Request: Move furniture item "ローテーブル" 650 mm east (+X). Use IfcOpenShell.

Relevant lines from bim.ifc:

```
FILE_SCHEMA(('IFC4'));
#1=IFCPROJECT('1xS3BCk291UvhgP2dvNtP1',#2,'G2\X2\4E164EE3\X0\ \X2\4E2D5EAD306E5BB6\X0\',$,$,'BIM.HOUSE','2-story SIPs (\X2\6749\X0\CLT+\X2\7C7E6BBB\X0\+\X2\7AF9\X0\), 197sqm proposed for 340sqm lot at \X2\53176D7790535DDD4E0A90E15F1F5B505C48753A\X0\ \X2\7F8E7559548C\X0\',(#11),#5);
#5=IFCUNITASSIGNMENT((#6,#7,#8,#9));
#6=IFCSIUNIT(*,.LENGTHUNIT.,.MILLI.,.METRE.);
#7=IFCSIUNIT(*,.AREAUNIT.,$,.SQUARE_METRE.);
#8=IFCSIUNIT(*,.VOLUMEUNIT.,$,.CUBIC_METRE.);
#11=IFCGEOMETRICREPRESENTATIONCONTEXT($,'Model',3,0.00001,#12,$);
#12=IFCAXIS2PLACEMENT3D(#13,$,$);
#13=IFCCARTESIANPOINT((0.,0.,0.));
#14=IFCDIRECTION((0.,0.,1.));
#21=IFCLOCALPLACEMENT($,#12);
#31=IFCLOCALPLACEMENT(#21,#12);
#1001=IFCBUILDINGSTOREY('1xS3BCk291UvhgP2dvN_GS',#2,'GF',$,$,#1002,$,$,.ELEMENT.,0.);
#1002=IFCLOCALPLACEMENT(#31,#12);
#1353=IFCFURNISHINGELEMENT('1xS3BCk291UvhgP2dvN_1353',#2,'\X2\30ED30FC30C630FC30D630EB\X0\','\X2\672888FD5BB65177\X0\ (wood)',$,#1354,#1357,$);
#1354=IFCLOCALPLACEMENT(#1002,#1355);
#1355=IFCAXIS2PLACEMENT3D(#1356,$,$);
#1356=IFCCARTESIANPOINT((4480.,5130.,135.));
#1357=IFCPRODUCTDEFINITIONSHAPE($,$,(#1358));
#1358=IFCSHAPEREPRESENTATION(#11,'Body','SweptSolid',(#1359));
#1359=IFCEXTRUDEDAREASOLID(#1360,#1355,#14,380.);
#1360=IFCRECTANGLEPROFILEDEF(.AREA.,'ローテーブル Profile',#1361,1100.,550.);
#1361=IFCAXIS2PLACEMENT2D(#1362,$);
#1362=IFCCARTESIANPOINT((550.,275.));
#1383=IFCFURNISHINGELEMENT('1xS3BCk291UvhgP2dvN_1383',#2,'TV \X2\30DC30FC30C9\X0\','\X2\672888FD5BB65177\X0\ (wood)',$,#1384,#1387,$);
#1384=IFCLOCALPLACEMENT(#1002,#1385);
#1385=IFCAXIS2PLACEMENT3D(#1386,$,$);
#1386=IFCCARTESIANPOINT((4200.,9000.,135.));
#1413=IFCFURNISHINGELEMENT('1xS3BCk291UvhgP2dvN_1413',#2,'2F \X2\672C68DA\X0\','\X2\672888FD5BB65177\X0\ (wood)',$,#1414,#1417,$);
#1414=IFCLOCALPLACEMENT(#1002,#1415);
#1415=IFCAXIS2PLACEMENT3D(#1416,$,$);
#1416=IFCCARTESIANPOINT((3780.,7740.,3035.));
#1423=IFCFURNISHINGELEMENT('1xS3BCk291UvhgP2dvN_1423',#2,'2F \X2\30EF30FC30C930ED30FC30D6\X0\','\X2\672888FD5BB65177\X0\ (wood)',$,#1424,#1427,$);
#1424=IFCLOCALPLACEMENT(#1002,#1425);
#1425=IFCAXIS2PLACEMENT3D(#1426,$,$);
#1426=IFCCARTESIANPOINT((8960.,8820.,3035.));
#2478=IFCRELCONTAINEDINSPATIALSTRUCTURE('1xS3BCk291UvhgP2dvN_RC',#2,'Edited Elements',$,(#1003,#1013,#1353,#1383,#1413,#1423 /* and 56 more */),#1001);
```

```python
import ifcopenshell
import ifcopenshell.api.geometry
import ifcopenshell.util.placement
import ifcopenshell.util.unit

model = ifcopenshell.open("bim.ifc")
unit_scale = ifcopenshell.util.unit.calculate_unit_scale(model)

item = model.by_guid("1xS3BCk291UvhgP2dvN_1353")
matrix = ifcopenshell.util.placement.get_local_placement(item.ObjectPlacement)
matrix[0, 3] += 0.65 / unit_scale
ifcopenshell.api.geometry.edit_object_placement(model, product=item, matrix=matrix, is_si=False)

print(ifcopenshell.util.placement.get_local_placement(item.ObjectPlacement).round(3) + 0.0)

model.write("bim_edited.ifc")
```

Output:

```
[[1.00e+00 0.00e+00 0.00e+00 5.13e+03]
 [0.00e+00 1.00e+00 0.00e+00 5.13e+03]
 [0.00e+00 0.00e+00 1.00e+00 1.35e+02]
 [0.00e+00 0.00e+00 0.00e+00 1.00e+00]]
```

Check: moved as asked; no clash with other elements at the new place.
